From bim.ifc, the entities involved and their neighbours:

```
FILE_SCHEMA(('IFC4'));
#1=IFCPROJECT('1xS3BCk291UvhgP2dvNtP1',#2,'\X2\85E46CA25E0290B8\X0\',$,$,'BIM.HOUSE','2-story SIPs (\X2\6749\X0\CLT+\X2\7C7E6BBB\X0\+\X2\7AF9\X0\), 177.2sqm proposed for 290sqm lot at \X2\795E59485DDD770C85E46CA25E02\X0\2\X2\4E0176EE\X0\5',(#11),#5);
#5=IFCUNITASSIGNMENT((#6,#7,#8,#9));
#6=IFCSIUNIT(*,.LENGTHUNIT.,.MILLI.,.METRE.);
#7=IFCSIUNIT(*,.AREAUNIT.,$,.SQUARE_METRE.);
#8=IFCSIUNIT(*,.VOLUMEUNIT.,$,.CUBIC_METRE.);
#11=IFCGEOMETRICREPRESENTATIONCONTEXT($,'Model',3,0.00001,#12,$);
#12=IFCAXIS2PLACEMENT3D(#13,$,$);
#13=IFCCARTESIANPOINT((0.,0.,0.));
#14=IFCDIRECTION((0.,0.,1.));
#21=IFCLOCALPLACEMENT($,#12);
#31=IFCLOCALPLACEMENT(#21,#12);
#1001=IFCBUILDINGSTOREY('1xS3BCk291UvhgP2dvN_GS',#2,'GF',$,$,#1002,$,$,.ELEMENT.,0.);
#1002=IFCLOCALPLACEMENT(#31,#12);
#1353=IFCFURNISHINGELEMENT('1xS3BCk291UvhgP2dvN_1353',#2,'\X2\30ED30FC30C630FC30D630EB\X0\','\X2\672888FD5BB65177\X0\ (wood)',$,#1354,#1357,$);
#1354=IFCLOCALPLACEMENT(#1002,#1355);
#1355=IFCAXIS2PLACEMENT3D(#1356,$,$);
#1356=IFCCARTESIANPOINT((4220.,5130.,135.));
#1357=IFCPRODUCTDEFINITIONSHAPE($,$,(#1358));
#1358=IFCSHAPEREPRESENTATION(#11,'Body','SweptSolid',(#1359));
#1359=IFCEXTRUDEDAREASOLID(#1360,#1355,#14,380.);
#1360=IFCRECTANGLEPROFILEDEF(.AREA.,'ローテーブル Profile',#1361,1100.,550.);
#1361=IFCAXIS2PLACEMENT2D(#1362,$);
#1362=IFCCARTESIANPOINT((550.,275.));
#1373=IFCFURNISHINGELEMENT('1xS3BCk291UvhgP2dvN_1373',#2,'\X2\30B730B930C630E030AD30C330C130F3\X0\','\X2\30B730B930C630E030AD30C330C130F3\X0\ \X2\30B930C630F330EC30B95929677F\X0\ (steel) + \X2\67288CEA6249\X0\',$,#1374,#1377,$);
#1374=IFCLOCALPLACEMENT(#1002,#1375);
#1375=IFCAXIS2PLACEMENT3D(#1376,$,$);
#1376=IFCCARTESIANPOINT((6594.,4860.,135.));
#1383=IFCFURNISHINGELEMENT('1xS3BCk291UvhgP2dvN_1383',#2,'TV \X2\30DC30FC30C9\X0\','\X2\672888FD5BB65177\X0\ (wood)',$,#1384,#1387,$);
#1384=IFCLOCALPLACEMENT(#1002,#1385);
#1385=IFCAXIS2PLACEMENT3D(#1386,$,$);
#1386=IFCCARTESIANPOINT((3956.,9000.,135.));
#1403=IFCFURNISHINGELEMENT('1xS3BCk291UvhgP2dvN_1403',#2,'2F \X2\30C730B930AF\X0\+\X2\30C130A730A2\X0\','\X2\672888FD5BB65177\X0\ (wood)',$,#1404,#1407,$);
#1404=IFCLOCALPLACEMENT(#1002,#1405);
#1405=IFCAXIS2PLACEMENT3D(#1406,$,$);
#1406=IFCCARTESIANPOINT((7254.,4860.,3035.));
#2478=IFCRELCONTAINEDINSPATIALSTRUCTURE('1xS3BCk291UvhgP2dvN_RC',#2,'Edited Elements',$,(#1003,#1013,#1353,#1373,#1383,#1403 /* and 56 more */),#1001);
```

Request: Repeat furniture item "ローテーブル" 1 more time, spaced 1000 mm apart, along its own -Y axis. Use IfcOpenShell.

```python
import ifcopenshell
import ifcopenshell.api.geometry
import ifcopenshell.api.root
import ifcopenshell.util.element
import ifcopenshell.util.placement
import ifcopenshell.util.unit

model = ifcopenshell.open("bim.ifc")
unit_scale = ifcopenshell.util.unit.calculate_unit_scale(model)


def reuse_history(source, copy):
    """copy_class also copies each property set's owner history, people and application; keep the originals."""
    for rel in copy.IsDefinedBy:
        if rel.is_a("IfcRelDefinesByProperties") and (history := rel.RelatingPropertyDefinition.OwnerHistory):
            rel.RelatingPropertyDefinition.OwnerHistory = source.OwnerHistory
            ifcopenshell.util.element.remove_deep2(model, history)


source = model.by_guid("1xS3BCk291UvhgP2dvN_1353")
base = ifcopenshell.util.placement.get_local_placement(source.ObjectPlacement)
step = -base[:3, 1] * 1 / unit_scale

for i in range(1, 2):
    copy = ifcopenshell.api.root.copy_class(model, product=source)
    copy.Representation = ifcopenshell.util.element.copy_deep(
        model, source.Representation, exclude=["IfcGeometricRepresentationContext", "IfcRepresentationMap"]
    )
    reuse_history(source, copy)
    matrix = base.copy()
    matrix[:3, 3] += i * step
    print("added at", matrix[:3, 3].round(3) + 0.0)
    ifcopenshell.api.geometry.edit_object_placement(model, product=copy, matrix=matrix, is_si=False)

model.write("bim_edited.ifc")
```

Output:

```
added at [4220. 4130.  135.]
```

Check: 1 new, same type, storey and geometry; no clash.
